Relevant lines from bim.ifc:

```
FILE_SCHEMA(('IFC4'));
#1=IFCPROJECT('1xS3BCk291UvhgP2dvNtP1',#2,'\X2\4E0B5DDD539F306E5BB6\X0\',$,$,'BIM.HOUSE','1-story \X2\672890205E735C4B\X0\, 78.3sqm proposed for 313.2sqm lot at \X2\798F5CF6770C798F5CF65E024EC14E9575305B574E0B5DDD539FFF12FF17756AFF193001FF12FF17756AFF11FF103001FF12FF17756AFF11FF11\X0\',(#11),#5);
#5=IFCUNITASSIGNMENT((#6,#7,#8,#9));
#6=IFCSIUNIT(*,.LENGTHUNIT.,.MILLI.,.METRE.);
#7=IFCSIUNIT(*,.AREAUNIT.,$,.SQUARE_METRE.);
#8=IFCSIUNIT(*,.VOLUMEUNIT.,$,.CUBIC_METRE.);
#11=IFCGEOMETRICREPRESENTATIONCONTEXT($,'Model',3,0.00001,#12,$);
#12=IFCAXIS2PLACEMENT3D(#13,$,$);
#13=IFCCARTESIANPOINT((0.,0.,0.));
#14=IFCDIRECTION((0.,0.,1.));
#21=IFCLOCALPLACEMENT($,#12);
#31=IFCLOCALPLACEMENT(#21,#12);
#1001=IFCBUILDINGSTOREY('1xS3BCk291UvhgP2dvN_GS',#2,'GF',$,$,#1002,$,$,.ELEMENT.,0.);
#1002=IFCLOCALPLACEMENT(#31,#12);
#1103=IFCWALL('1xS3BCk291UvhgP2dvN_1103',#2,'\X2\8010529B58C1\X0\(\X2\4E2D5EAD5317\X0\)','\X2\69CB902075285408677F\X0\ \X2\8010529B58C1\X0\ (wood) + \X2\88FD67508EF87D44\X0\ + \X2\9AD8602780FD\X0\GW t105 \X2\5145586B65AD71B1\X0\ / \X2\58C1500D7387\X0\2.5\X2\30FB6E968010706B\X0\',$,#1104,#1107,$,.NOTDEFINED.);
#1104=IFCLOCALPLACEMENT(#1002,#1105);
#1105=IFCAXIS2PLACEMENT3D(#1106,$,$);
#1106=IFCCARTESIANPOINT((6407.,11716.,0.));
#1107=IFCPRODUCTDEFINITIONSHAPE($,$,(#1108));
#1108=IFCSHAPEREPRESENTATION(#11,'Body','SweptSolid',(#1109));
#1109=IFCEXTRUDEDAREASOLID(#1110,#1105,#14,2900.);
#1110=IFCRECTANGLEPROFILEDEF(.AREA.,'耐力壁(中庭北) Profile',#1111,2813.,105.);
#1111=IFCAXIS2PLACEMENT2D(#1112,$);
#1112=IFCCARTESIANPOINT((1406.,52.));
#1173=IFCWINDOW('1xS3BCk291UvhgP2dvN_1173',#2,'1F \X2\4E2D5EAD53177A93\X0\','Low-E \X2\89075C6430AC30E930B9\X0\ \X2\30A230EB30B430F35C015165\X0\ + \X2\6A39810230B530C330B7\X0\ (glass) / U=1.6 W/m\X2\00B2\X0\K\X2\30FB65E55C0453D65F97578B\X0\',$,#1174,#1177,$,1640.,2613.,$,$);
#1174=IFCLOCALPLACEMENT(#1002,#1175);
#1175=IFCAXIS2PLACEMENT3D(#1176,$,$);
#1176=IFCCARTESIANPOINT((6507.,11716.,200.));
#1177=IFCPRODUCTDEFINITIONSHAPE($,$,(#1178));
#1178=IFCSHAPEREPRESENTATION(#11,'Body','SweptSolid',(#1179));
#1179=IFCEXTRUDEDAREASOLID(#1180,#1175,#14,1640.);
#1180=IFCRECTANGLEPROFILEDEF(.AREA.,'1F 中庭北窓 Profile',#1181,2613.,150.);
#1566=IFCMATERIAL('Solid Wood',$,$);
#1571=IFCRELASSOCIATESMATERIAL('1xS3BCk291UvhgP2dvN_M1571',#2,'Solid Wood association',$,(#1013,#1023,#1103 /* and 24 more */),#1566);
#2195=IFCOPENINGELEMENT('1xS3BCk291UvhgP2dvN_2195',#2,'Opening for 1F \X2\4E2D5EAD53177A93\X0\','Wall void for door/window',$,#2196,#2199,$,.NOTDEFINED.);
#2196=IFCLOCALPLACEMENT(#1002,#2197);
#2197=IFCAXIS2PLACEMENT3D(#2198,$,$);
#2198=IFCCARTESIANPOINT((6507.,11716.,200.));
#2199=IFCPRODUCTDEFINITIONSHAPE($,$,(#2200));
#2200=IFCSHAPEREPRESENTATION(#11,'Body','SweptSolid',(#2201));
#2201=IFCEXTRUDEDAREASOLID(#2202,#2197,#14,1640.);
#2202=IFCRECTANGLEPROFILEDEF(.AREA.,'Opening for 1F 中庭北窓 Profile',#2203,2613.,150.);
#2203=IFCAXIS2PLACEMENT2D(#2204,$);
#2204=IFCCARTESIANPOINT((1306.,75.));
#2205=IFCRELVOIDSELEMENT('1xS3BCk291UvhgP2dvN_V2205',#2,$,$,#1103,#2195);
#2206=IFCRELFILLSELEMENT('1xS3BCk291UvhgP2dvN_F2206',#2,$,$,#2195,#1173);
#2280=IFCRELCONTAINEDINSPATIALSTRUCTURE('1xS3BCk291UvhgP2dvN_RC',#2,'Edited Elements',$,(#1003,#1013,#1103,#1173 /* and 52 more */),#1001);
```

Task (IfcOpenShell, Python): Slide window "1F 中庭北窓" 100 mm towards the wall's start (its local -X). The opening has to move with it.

```python
import ifcopenshell
import ifcopenshell.api.geometry
import ifcopenshell.util.placement
import ifcopenshell.util.unit

model = ifcopenshell.open("bim.ifc")
unit_scale = ifcopenshell.util.unit.calculate_unit_scale(model)

window = model.by_guid("1xS3BCk291UvhgP2dvN_1173")
opening = window.FillsVoids[0].RelatingOpeningElement
wall = opening.VoidsElements[0].RelatingBuildingElement

wall_matrix = ifcopenshell.util.placement.get_local_placement(wall.ObjectPlacement)
shift = wall_matrix[:3, 0] * -0.1 / unit_scale
before = ifcopenshell.util.placement.get_local_placement(window.ObjectPlacement)[:3, 3].copy()

# The window is not placed relative to its opening, so move both.
for product in (opening, window):
    matrix = ifcopenshell.util.placement.get_local_placement(product.ObjectPlacement)
    matrix[:3, 3] += shift
    ifcopenshell.api.geometry.edit_object_placement(model, product=product, matrix=matrix, is_si=False)

after = ifcopenshell.util.placement.get_local_placement(window.ObjectPlacement)[:3, 3]
print("window moved by", (after - before).round(3) + 0.0)

model.write("bim-out.ifc")
```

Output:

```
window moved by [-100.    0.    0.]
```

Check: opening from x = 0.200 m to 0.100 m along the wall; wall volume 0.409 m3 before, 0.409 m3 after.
